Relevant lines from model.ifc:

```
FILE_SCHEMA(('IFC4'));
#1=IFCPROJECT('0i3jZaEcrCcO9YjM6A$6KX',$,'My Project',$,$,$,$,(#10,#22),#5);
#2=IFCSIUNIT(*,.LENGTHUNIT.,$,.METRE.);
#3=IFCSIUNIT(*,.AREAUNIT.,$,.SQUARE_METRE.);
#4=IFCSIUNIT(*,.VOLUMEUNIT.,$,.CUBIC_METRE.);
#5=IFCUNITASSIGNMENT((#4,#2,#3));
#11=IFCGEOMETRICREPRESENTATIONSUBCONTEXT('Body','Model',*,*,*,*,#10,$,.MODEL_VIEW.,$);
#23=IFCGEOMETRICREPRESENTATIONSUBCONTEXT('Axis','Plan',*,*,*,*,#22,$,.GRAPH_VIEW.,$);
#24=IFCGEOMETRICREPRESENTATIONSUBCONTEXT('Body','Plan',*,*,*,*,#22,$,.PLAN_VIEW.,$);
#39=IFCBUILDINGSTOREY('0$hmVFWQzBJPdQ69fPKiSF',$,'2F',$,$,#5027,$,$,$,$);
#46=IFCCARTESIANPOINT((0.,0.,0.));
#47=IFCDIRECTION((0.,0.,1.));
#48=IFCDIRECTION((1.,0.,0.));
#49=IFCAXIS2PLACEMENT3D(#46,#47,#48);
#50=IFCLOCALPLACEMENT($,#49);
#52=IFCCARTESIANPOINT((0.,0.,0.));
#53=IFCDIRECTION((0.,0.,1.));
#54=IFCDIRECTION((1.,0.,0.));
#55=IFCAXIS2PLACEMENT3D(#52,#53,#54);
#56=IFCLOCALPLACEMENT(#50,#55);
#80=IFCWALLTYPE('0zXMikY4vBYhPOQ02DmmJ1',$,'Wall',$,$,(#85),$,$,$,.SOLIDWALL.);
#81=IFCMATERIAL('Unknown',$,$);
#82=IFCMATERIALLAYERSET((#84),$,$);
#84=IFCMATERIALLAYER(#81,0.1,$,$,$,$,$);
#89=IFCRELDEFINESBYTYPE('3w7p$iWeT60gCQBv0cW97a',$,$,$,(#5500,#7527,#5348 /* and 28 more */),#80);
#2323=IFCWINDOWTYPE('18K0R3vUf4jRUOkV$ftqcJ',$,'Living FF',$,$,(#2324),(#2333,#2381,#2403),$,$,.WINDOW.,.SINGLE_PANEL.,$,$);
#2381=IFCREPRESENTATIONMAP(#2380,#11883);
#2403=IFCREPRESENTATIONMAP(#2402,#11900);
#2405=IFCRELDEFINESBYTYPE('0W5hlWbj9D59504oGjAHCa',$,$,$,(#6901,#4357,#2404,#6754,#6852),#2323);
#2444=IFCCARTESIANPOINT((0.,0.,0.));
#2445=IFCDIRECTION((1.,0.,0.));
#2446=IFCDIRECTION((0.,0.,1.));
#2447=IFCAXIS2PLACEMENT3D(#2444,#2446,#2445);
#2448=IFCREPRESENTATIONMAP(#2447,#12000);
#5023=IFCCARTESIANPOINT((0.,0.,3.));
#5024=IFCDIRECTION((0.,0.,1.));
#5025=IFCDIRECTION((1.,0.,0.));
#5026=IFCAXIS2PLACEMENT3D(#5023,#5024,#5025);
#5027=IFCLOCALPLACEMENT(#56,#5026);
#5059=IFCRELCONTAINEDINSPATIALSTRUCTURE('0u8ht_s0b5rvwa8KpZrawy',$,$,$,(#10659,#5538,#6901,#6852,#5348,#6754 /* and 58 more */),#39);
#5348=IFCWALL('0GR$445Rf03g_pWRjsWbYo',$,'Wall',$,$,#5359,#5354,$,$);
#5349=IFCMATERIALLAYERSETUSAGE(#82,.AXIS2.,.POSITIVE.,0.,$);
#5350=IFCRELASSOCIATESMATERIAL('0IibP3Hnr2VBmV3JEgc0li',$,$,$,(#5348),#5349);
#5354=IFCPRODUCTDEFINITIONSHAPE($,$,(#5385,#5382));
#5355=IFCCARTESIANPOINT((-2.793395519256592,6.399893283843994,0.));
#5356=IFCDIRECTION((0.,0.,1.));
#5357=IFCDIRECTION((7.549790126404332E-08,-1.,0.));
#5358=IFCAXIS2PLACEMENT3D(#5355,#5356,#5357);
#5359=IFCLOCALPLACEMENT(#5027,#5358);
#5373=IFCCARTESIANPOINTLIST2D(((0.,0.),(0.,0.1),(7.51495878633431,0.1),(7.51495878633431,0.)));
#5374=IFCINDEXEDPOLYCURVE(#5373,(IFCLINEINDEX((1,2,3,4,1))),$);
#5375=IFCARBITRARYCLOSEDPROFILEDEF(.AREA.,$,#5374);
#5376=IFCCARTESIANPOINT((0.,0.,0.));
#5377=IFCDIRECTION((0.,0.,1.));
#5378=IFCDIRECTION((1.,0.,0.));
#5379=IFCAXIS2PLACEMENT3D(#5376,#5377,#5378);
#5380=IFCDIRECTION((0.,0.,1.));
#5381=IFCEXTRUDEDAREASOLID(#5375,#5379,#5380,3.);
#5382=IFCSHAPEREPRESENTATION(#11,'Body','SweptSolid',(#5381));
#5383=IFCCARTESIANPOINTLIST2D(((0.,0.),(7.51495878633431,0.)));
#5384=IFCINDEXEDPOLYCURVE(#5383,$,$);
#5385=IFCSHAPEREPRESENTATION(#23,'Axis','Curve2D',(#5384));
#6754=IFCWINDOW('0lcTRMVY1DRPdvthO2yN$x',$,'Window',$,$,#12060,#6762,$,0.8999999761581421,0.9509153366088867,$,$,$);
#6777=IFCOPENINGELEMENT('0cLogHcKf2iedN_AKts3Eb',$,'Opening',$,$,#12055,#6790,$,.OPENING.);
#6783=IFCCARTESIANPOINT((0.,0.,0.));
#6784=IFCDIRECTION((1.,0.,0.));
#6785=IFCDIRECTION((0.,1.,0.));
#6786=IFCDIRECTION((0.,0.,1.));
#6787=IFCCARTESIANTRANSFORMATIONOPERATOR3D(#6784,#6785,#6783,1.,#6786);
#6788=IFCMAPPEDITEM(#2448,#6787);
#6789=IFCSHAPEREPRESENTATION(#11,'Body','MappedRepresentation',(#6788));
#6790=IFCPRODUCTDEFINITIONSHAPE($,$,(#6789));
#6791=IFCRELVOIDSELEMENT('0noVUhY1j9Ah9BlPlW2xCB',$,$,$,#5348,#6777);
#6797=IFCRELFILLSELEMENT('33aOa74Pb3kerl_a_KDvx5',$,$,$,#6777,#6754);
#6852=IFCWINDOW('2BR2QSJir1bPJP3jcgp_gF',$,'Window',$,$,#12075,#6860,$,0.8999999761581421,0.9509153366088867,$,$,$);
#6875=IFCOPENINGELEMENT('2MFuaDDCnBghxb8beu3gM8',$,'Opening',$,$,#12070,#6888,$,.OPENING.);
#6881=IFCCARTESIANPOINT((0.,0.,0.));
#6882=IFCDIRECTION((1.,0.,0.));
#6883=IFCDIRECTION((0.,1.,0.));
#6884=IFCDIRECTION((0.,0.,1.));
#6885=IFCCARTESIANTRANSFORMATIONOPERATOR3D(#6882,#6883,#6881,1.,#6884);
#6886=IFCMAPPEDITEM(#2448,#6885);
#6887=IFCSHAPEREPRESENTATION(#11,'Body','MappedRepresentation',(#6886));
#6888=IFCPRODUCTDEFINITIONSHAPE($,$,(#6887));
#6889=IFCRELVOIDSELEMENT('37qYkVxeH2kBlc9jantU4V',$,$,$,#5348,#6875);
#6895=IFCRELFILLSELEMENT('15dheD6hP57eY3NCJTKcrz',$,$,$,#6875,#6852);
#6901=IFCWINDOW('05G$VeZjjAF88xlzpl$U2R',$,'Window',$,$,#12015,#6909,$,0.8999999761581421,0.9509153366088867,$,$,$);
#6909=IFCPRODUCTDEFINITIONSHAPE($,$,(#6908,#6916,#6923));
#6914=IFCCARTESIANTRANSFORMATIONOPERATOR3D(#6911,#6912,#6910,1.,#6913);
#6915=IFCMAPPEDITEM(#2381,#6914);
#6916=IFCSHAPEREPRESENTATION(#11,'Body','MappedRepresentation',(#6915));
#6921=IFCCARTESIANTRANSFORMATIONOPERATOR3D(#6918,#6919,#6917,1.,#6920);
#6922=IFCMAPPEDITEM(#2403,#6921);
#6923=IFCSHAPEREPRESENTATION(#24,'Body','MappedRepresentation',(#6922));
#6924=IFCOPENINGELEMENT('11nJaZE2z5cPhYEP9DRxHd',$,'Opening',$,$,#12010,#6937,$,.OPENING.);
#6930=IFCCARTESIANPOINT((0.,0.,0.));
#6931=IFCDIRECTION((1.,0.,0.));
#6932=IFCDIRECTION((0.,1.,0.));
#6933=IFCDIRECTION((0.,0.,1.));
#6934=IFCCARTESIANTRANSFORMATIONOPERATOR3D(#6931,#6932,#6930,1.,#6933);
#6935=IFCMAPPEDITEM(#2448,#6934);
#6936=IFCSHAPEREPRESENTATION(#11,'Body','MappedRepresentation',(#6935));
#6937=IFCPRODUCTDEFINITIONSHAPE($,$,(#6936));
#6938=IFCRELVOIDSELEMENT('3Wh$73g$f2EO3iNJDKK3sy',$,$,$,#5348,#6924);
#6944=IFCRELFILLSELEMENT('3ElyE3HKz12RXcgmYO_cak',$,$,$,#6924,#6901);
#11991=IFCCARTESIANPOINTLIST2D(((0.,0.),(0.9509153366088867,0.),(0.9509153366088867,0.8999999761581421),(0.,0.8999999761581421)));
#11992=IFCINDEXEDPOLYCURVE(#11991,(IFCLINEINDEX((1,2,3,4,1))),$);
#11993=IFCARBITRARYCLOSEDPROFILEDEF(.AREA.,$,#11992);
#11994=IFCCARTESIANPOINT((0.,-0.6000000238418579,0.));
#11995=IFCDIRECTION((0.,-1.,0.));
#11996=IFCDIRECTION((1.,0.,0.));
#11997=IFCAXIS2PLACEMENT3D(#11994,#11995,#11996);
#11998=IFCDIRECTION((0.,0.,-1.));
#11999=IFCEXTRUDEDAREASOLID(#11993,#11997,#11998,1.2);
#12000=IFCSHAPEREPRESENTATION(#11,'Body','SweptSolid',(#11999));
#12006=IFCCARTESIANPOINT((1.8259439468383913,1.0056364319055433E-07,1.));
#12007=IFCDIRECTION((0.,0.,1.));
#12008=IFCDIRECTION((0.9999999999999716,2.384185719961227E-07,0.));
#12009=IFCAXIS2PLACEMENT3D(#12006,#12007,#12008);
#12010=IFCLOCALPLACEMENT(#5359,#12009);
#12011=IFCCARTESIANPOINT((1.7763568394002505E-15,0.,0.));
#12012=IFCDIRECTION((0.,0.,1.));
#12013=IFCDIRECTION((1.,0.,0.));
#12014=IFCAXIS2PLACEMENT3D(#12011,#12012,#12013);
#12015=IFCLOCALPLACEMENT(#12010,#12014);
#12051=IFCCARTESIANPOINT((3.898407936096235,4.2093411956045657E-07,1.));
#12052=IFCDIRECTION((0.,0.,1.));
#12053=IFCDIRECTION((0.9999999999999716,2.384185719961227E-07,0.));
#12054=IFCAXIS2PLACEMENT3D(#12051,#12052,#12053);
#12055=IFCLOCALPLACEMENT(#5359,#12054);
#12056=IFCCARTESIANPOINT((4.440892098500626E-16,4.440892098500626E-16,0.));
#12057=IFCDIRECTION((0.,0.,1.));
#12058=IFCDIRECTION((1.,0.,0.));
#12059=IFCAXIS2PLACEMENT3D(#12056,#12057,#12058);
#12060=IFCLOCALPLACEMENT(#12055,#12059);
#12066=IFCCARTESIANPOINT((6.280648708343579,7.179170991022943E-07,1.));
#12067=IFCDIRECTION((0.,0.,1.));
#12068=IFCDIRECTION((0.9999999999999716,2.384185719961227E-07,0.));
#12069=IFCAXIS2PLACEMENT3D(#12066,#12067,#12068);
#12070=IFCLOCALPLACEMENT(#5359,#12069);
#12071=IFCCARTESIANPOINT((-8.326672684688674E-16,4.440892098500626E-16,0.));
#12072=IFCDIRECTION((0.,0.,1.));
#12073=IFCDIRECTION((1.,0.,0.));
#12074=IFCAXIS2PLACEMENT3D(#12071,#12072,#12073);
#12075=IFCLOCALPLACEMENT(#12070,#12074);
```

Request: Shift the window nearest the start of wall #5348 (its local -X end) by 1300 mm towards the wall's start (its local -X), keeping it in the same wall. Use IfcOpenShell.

```python
import ifcopenshell
import ifcopenshell.api.geometry
import ifcopenshell.util.placement
import ifcopenshell.util.unit

model = ifcopenshell.open("model.ifc")
unit_scale = ifcopenshell.util.unit.calculate_unit_scale(model)

window = model.by_guid("05G$VeZjjAF88xlzpl$U2R")
opening = window.FillsVoids[0].RelatingOpeningElement
wall = opening.VoidsElements[0].RelatingBuildingElement

wall_matrix = ifcopenshell.util.placement.get_local_placement(wall.ObjectPlacement)
shift = wall_matrix[:3, 0] * -1.3 / unit_scale
before = ifcopenshell.util.placement.get_local_placement(window.ObjectPlacement)[:3, 3].copy()

# The window is placed relative to its opening, so it follows when the opening moves.
matrix = ifcopenshell.util.placement.get_local_placement(opening.ObjectPlacement)
matrix[:3, 3] += shift
ifcopenshell.api.geometry.edit_object_placement(
    model, product=opening, matrix=matrix, is_si=False, should_transform_children=True
)

after = ifcopenshell.util.placement.get_local_placement(window.ObjectPlacement)[:3, 3]
print("window moved by", (after - before).round(3) + 0.0)

model.write("model_v2.ifc")
```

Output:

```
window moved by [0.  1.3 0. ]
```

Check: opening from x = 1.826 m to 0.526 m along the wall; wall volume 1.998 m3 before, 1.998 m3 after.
